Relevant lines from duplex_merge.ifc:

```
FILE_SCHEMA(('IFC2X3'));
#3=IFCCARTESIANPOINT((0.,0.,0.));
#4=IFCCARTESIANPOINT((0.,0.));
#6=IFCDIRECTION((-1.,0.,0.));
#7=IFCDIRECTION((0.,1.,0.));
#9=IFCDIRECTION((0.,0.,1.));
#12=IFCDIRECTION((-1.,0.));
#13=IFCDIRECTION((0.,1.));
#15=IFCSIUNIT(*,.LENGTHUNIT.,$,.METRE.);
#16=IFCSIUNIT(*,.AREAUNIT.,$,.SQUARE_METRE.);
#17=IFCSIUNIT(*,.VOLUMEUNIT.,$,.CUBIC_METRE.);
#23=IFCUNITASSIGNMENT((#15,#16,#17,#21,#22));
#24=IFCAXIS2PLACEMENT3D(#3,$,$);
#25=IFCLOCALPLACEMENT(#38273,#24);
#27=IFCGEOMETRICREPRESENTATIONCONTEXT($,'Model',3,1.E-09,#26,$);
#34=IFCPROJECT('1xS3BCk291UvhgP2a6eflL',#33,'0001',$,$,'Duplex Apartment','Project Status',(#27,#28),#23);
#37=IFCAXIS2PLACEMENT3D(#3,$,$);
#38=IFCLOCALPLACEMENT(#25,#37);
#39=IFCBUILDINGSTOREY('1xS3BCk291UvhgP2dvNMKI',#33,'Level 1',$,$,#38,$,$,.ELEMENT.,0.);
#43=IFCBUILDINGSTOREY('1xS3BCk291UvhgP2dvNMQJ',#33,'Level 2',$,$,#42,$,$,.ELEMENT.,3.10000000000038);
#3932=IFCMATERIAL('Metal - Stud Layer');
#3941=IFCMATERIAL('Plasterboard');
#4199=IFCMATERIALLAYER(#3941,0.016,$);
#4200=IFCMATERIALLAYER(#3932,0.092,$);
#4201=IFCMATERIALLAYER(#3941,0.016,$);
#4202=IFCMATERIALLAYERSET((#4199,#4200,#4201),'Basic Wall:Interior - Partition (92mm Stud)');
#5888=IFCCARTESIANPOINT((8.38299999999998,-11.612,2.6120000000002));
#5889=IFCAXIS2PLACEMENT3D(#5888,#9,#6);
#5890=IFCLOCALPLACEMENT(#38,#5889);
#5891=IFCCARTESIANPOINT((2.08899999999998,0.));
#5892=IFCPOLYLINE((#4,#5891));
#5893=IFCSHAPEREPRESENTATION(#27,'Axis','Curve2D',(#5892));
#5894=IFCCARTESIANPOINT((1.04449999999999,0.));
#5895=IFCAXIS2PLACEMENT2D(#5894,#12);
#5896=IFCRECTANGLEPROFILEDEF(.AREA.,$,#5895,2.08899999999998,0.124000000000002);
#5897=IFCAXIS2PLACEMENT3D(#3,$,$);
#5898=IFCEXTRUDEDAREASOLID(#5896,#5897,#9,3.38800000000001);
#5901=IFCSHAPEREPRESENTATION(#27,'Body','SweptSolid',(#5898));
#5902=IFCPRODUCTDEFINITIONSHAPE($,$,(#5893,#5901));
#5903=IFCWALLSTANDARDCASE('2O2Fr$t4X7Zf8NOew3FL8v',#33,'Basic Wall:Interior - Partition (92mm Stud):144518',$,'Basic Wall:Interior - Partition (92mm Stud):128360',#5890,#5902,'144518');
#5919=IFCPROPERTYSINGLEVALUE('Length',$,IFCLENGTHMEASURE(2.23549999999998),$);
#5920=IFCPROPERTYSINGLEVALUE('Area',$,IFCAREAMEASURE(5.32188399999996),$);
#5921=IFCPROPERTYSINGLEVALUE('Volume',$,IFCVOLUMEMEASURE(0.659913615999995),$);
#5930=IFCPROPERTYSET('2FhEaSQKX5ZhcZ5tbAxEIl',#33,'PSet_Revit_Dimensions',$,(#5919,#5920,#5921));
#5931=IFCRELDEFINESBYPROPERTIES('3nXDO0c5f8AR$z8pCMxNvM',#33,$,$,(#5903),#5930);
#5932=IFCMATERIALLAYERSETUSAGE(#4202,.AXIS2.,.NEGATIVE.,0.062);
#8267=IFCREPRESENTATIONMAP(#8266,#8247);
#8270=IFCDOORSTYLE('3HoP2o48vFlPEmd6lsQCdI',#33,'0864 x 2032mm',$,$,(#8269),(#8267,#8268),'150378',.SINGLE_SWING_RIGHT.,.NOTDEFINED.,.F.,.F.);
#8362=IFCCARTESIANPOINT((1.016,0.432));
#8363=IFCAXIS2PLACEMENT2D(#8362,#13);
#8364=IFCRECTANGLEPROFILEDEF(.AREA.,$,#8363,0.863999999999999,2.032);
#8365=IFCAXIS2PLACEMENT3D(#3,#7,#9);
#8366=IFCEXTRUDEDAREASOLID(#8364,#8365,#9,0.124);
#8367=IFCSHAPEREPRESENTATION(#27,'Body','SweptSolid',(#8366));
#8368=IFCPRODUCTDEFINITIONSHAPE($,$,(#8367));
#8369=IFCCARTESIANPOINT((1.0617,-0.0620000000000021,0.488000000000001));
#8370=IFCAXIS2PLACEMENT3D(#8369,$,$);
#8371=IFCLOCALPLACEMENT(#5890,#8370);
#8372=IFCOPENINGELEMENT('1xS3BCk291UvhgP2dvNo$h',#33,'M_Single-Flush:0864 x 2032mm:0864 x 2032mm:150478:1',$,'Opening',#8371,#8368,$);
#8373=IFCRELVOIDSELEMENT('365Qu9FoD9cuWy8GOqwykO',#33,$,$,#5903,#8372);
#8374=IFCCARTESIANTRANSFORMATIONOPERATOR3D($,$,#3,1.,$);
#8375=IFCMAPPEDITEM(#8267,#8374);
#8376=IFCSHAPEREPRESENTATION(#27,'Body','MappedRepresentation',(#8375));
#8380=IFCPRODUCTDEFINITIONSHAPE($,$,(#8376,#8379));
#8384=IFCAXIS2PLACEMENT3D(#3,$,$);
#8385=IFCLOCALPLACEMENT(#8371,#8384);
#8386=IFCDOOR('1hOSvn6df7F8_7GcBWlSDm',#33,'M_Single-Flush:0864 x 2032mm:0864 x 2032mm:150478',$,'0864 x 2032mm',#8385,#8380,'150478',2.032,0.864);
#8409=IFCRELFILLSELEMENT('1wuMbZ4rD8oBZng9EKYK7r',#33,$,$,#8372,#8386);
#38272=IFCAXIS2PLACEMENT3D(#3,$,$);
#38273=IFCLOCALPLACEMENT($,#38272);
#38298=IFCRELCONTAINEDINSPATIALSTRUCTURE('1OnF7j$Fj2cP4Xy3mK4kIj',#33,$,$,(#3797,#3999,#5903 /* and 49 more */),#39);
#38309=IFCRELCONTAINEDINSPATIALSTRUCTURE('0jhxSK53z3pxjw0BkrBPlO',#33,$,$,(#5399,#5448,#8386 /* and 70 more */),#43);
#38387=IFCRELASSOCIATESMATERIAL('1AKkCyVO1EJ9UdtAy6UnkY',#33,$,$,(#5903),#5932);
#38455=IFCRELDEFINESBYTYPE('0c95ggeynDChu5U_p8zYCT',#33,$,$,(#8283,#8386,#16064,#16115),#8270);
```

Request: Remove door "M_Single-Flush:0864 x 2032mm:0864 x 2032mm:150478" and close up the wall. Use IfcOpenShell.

```python
import ifcopenshell
import ifcopenshell.api.feature
import ifcopenshell.api.pset
import ifcopenshell.api.root
import ifcopenshell.geom
import ifcopenshell.util.element
import ifcopenshell.util.shape
import ifcopenshell.util.unit

model = ifcopenshell.open("duplex_merge.ifc")
area_scale = ifcopenshell.util.unit.calculate_unit_scale(model, "AREAUNIT")
volume_scale = ifcopenshell.util.unit.calculate_unit_scale(model, "VOLUMEUNIT")
settings = ifcopenshell.geom.settings()


def volume(element):
    """Net volume in cubic metres, openings subtracted."""
    shape = ifcopenshell.geom.create_shape(settings, element)
    return ifcopenshell.util.shape.get_volume(shape.geometry)


door = model.by_guid("1hOSvn6df7F8_7GcBWlSDm")
opening = door.FillsVoids[0].RelatingOpeningElement
wall = opening.VoidsElements[0].RelatingBuildingElement
before = volume(wall)

ifcopenshell.api.root.remove_product(model, product=door)
ifcopenshell.api.feature.remove_feature(model, feature=opening)

after = volume(wall)
thickness = 0.124  # wall thickness in metres

# Update the wall's stored quantities.
pset = model.by_id(ifcopenshell.util.element.get_pset(wall, "PSet_Revit_Dimensions", should_inherit=False)["id"])
ifcopenshell.api.pset.edit_pset(model, pset=pset, properties={
    "Area": model.create_entity("IfcAreaMeasure", after / thickness / area_scale),
    "Volume": model.create_entity("IfcVolumeMeasure", after / volume_scale),
})

print(f"wall volume {before:.3f} -> {after:.3f} m3")

model.write("duplex_merge_v2.ifc")
```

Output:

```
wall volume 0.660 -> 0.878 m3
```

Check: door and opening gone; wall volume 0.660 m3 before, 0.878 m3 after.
